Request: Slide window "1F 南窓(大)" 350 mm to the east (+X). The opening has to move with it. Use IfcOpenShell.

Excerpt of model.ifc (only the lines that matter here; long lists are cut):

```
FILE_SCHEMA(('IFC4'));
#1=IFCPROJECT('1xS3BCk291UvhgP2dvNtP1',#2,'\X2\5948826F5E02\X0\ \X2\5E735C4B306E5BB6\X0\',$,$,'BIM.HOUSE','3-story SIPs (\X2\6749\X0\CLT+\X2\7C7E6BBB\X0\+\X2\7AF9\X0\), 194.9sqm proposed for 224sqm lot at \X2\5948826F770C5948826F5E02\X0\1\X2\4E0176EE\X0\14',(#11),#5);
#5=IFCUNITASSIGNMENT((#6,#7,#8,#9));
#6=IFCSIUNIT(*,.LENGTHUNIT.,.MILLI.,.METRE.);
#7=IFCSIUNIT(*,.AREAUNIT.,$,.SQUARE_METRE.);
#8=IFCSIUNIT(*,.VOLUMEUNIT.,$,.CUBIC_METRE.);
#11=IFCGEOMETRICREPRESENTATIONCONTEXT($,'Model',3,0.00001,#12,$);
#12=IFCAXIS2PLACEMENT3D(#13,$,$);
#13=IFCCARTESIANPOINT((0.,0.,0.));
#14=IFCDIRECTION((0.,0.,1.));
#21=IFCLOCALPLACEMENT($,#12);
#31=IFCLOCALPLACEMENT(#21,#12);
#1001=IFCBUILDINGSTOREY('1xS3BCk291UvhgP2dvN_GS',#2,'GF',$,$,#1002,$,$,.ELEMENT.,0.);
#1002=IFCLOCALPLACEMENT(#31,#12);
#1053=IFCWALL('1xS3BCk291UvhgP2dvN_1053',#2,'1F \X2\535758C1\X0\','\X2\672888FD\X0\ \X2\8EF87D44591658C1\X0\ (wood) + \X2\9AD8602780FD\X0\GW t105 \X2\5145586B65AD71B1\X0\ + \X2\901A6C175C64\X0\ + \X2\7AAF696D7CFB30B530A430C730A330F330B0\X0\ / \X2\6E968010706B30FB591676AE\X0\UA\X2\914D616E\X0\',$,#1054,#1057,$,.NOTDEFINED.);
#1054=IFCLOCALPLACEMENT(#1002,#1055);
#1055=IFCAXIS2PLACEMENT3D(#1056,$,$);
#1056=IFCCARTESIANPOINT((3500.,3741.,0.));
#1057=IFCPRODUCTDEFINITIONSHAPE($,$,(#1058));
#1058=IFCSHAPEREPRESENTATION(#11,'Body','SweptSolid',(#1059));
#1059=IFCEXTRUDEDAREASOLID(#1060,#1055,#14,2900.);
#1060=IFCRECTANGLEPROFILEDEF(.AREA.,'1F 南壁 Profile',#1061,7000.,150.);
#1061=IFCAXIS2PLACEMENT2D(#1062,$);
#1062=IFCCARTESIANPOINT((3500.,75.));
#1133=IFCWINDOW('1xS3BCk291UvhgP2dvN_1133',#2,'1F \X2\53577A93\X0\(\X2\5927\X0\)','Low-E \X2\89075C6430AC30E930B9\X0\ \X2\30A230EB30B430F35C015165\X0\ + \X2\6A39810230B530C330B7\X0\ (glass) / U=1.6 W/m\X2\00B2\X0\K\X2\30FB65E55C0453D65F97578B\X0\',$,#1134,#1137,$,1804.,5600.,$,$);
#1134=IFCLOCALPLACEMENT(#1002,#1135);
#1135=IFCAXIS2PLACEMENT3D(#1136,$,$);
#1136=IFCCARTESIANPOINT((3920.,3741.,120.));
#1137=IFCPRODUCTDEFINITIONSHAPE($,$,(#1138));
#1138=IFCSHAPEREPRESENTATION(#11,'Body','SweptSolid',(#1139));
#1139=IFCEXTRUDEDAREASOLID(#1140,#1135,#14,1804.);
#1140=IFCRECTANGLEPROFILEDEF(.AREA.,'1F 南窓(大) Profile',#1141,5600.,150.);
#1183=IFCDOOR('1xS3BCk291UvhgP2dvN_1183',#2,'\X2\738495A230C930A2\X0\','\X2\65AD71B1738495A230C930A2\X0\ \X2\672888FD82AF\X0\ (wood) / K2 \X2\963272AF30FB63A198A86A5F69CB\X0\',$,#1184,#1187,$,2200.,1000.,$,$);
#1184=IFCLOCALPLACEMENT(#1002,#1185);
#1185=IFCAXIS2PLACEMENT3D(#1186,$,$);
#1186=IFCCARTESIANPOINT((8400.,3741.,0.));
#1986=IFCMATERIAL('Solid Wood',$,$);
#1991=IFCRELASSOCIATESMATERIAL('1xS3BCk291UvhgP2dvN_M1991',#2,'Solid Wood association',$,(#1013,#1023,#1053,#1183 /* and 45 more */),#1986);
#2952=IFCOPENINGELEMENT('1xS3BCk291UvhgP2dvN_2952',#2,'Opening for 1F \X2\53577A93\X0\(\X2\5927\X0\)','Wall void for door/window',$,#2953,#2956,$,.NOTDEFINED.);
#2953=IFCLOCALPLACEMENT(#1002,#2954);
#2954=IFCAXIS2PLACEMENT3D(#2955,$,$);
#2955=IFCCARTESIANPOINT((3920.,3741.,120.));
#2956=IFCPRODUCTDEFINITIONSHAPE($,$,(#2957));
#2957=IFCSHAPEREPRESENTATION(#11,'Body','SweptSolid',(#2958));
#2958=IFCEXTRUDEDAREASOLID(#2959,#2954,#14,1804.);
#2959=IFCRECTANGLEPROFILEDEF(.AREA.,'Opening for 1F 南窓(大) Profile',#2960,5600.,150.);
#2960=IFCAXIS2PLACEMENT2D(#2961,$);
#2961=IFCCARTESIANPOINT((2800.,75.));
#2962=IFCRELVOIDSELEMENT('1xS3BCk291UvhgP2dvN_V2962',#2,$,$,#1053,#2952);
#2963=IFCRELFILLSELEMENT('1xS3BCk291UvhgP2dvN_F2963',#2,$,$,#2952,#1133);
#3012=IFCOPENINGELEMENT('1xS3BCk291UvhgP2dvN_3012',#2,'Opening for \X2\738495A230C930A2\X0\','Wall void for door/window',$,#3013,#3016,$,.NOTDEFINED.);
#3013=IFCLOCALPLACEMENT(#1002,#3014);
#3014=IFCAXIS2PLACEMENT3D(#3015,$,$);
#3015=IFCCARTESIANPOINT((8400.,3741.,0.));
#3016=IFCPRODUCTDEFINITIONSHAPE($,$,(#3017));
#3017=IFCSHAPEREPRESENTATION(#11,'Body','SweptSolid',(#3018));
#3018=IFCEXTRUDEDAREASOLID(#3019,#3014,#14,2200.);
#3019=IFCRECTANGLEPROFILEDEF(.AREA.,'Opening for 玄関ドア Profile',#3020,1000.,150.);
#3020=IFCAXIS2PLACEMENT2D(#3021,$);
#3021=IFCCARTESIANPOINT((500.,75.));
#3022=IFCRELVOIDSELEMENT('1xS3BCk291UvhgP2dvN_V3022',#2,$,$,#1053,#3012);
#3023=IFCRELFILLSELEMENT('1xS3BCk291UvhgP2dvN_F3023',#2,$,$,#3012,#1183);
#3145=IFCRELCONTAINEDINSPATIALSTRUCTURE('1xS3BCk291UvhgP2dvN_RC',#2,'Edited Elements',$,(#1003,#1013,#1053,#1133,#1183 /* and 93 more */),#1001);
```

```python
import ifcopenshell
import ifcopenshell.api.geometry
import ifcopenshell.util.placement
import ifcopenshell.util.unit

model = ifcopenshell.open("model.ifc")
unit_scale = ifcopenshell.util.unit.calculate_unit_scale(model)

window = model.by_guid("1xS3BCk291UvhgP2dvN_1133")
opening = window.FillsVoids[0].RelatingOpeningElement
wall = opening.VoidsElements[0].RelatingBuildingElement

wall_matrix = ifcopenshell.util.placement.get_local_placement(wall.ObjectPlacement)
shift = wall_matrix[:3, 0] * 0.35 / unit_scale
before = ifcopenshell.util.placement.get_local_placement(window.ObjectPlacement)[:3, 3].copy()

# The window is not placed relative to its opening, so move both.
for product in (opening, window):
    matrix = ifcopenshell.util.placement.get_local_placement(product.ObjectPlacement)
    matrix[:3, 3] += shift
    ifcopenshell.api.geometry.edit_object_placement(model, product=product, matrix=matrix, is_si=False)

after = ifcopenshell.util.placement.get_local_placement(window.ObjectPlacement)[:3, 3]
print("window moved by", (after - before).round(3) + 0.0)

model.write("model_rev.ifc")
```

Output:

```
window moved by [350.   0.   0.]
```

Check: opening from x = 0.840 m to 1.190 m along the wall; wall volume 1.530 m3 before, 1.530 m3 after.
